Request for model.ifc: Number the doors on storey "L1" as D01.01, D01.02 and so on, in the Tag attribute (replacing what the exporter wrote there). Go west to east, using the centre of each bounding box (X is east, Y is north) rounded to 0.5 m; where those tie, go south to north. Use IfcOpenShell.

First a look at what the model holds.

```python
import ifcopenshell
import ifcopenshell.util.element
import ifcopenshell.util.placement

model = ifcopenshell.open("model.ifc")
print(model.schema)
storey = next(s for s in model.by_type("IfcBuildingStorey") if s.Name == "L1")
doors = [e for e in ifcopenshell.util.element.get_decomposition(storey) if e.is_a("IfcDoor")]
for e in sorted(doors, key=lambda e: e.id()):
    origin = ifcopenshell.util.placement.get_local_placement(e.ObjectPlacement)[:3, 3]
    print(e.id(), e.Tag, e.Name, origin.round(2) + 0.0, sep=" | ")
```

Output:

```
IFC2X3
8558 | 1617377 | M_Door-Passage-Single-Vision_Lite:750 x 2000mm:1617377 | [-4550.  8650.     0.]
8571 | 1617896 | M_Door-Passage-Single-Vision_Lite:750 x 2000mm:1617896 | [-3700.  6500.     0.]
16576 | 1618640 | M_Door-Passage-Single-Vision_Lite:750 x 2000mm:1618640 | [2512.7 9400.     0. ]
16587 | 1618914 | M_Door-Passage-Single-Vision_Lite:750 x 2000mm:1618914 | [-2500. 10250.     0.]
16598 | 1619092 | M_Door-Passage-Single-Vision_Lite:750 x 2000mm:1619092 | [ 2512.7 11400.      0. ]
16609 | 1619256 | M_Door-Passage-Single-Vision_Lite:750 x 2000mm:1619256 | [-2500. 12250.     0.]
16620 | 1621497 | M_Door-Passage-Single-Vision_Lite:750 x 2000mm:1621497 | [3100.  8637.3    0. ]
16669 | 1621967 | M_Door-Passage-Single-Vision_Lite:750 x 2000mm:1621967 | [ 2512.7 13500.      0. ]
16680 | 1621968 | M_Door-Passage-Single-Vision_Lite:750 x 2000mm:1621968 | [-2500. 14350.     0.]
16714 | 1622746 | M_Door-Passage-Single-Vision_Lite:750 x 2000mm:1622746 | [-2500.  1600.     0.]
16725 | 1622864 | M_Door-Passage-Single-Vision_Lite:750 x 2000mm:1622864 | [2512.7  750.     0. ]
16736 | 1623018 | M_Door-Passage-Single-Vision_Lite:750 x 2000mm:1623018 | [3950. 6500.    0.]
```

```python
import ifcopenshell
import ifcopenshell.geom
import ifcopenshell.util.element
import ifcopenshell.util.shape

model = ifcopenshell.open("model.ifc")
settings = ifcopenshell.geom.settings()
settings.set("use-world-coords", True)


def centre(element):
    shape = ifcopenshell.geom.create_shape(settings, element)
    return ifcopenshell.util.shape.get_bbox_centroid(shape.geometry)


storey = next(s for s in model.by_type("IfcBuildingStorey") if s.Name == "L1")
doors = [e for e in ifcopenshell.util.element.get_decomposition(storey) if e.is_a("IfcDoor")]

# Insertion points can sit at a corner or the storey origin, so sort by the geometry (in metres).
centres = {e: centre(e) for e in doors}
doors.sort(key=lambda e: (round(centres[e][0] / 0.5), centres[e][1]))

for i, e in enumerate(doors, start=1):
    number = f"D01.{i:02d}"
    e.Tag = number
    print(e.id(), number)

model.write("model_updated.ifc")
```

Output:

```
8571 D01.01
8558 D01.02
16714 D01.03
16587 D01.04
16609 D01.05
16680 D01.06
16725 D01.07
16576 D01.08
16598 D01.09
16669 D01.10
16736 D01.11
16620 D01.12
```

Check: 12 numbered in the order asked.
